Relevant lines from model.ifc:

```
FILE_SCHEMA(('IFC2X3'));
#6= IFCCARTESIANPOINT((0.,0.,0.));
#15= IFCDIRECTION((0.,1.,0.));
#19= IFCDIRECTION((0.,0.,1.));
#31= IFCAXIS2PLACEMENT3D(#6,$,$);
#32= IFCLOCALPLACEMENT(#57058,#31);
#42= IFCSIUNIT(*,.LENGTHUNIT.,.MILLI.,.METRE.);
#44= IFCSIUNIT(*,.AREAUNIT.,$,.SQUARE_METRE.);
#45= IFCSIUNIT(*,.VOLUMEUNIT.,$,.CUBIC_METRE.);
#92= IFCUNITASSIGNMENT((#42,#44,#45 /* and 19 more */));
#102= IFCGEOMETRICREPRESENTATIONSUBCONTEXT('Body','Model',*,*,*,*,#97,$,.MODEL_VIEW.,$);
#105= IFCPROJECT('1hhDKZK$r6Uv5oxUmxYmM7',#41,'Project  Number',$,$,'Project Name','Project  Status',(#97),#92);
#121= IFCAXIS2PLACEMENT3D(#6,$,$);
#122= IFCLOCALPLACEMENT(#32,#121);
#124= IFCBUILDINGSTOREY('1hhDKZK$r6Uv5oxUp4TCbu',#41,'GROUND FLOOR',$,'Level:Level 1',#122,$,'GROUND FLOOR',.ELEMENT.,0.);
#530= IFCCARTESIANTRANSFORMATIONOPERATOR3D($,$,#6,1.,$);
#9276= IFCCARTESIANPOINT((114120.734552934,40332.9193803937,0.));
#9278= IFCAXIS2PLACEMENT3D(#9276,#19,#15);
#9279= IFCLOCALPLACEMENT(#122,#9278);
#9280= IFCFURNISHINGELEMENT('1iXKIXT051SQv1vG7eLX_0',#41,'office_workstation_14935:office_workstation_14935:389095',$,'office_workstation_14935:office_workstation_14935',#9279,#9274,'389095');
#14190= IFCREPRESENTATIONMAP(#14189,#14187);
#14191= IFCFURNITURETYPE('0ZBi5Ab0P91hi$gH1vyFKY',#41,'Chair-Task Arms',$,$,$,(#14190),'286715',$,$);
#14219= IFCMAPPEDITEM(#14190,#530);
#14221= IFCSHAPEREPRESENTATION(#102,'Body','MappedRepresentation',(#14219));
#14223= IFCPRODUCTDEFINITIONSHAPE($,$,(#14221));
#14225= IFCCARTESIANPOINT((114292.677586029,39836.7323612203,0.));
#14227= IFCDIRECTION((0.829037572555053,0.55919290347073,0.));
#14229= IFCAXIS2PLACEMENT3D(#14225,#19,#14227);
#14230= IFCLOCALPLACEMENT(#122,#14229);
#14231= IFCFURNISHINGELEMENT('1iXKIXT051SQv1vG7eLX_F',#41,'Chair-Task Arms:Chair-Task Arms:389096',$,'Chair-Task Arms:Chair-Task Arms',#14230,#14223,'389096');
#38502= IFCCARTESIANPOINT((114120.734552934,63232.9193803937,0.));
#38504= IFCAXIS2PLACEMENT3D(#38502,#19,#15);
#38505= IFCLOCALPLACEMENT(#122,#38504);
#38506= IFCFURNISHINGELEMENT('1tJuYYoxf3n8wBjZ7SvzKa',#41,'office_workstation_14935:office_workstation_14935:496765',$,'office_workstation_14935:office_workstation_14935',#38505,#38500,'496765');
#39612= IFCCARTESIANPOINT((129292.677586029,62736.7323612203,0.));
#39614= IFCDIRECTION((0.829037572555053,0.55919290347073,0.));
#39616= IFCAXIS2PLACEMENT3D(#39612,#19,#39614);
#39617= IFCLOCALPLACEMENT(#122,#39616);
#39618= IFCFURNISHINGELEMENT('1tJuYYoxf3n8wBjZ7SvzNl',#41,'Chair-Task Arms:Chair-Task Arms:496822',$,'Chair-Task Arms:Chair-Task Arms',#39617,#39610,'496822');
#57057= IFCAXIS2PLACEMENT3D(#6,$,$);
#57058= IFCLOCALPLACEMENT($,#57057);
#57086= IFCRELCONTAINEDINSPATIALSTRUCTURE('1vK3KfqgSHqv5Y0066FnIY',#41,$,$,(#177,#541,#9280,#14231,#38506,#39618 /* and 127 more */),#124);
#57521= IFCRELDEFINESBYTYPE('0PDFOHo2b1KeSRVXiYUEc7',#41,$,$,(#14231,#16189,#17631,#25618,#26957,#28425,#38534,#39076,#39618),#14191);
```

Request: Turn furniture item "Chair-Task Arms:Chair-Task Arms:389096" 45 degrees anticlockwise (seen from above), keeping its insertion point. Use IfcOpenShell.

```python
import ifcopenshell
import ifcopenshell.api.geometry
import ifcopenshell.util.placement

model = ifcopenshell.open("model.ifc")

item = model.by_guid("1iXKIXT051SQv1vG7eLX_F")
matrix = ifcopenshell.util.placement.get_local_placement(item.ObjectPlacement)
matrix = matrix @ ifcopenshell.util.placement.rotation(45, "Z")
ifcopenshell.api.geometry.edit_object_placement(model, product=item, matrix=matrix, is_si=False)

print(ifcopenshell.util.placement.get_local_placement(item.ObjectPlacement).round(3) + 0.0)

model.write("model_rev.ifc")
```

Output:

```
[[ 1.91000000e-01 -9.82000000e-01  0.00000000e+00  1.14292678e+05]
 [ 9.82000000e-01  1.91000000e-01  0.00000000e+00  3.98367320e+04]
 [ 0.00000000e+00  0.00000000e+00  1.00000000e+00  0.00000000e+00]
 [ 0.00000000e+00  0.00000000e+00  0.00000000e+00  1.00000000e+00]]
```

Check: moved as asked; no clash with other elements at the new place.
